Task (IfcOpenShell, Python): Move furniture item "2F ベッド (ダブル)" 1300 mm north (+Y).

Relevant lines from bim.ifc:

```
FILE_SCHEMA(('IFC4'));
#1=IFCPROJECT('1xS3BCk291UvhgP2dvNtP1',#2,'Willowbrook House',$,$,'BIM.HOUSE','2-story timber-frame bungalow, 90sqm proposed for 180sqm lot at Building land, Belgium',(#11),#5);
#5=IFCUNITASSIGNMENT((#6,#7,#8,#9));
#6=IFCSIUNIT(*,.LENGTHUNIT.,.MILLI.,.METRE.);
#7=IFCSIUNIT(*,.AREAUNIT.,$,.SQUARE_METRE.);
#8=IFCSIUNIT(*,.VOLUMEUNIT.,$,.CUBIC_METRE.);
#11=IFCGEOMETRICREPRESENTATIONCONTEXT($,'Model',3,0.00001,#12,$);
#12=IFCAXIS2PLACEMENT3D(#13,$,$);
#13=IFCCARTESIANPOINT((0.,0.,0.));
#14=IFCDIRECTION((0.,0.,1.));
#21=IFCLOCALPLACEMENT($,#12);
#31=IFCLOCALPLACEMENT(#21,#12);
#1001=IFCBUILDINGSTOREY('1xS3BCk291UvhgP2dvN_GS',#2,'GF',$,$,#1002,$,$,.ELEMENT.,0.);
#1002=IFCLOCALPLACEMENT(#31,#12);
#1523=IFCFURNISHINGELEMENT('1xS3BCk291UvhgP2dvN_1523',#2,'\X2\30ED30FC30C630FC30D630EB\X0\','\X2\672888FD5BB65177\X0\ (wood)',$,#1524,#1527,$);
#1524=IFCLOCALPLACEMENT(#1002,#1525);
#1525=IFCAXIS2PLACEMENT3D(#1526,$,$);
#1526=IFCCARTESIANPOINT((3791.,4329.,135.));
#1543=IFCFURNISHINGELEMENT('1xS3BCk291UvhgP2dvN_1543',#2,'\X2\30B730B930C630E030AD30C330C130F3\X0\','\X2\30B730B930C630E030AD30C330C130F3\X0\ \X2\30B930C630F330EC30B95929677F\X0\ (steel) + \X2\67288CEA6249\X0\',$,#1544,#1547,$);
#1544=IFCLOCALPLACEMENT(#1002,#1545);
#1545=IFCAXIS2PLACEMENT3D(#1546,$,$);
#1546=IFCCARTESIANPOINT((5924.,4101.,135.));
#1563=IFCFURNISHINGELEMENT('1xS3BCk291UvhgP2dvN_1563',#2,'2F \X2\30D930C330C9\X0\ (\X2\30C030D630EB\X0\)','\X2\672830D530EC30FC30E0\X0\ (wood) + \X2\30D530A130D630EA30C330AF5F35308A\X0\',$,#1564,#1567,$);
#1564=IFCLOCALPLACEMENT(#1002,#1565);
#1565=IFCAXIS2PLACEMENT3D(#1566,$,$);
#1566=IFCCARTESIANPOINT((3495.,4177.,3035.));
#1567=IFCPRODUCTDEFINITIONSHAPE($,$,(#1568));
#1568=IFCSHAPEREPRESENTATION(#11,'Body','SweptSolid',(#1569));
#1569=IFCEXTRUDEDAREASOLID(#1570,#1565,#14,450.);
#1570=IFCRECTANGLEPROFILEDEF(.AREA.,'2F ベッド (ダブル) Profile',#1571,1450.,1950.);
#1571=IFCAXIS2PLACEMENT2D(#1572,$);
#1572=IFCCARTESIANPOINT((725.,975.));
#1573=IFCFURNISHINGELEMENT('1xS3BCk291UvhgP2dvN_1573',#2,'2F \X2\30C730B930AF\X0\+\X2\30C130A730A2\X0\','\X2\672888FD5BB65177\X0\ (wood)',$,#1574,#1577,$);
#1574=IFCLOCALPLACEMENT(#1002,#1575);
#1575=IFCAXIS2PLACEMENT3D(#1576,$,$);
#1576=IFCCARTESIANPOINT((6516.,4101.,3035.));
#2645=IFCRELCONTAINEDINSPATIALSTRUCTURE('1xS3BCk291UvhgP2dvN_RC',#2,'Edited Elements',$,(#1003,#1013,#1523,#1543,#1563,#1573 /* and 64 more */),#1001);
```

```python
import ifcopenshell
import ifcopenshell.api.geometry
import ifcopenshell.util.placement
import ifcopenshell.util.unit

model = ifcopenshell.open("bim.ifc")
unit_scale = ifcopenshell.util.unit.calculate_unit_scale(model)

item = model.by_guid("1xS3BCk291UvhgP2dvN_1563")
matrix = ifcopenshell.util.placement.get_local_placement(item.ObjectPlacement)
matrix[1, 3] += 1.3 / unit_scale
ifcopenshell.api.geometry.edit_object_placement(model, product=item, matrix=matrix, is_si=False)

print(ifcopenshell.util.placement.get_local_placement(item.ObjectPlacement).round(3) + 0.0)

model.write("bim_rev.ifc")
```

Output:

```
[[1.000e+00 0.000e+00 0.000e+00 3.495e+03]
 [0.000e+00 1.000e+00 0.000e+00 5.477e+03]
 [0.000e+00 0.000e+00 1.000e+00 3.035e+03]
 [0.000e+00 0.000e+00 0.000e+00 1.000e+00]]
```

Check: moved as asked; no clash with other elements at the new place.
